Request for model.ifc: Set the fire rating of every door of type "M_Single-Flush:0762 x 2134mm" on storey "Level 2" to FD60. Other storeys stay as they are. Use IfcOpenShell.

First a look at what the model holds.

```python
import ifcopenshell
import ifcopenshell.util.element

model = ifcopenshell.open("model.ifc")
print(model.schema)
storey = next(s for s in model.by_type("IfcBuildingStorey") if s.Name == "Level 2")
doors = [e for e in ifcopenshell.util.element.get_decomposition(storey) if e.is_a("IfcDoor")]
seen = {}
for e in doors:
    element_type = ifcopenshell.util.element.get_type(e)
    key = (element_type.Name if element_type != e and element_type else None, ifcopenshell.util.element.get_pset(e, "Pset_DoorCommon", "FireRating"))
    seen[key] = seen.get(key, 0) + 1
for (name, value), count in sorted(seen.items(), key=str):
    print(count, "x", name, "|", value)
```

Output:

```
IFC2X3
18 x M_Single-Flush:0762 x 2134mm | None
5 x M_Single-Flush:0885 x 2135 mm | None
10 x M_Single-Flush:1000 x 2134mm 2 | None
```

```python
import ifcopenshell
import ifcopenshell.api.pset
import ifcopenshell.util.element

model = ifcopenshell.open("model.ifc")

storey = next(s for s in model.by_type("IfcBuildingStorey") if s.Name == "Level 2")
doors = [e for e in ifcopenshell.util.element.get_decomposition(storey) if e.is_a("IfcDoor")]

count = 0
for e in doors:
    element_type = ifcopenshell.util.element.get_type(e)
    if element_type in (None, e) or element_type.Name != "M_Single-Flush:0762 x 2134mm":
        continue
    # add_pset returns the element's existing set when there is one.
    pset = ifcopenshell.api.pset.add_pset(model, product=e, name="Pset_DoorCommon")
    ifcopenshell.api.pset.edit_pset(model, pset=pset, properties={"FireRating": "FD60"})
    count += 1

print(count, "doors updated")

model.write("model_edited.ifc")
```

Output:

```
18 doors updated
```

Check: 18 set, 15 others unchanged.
